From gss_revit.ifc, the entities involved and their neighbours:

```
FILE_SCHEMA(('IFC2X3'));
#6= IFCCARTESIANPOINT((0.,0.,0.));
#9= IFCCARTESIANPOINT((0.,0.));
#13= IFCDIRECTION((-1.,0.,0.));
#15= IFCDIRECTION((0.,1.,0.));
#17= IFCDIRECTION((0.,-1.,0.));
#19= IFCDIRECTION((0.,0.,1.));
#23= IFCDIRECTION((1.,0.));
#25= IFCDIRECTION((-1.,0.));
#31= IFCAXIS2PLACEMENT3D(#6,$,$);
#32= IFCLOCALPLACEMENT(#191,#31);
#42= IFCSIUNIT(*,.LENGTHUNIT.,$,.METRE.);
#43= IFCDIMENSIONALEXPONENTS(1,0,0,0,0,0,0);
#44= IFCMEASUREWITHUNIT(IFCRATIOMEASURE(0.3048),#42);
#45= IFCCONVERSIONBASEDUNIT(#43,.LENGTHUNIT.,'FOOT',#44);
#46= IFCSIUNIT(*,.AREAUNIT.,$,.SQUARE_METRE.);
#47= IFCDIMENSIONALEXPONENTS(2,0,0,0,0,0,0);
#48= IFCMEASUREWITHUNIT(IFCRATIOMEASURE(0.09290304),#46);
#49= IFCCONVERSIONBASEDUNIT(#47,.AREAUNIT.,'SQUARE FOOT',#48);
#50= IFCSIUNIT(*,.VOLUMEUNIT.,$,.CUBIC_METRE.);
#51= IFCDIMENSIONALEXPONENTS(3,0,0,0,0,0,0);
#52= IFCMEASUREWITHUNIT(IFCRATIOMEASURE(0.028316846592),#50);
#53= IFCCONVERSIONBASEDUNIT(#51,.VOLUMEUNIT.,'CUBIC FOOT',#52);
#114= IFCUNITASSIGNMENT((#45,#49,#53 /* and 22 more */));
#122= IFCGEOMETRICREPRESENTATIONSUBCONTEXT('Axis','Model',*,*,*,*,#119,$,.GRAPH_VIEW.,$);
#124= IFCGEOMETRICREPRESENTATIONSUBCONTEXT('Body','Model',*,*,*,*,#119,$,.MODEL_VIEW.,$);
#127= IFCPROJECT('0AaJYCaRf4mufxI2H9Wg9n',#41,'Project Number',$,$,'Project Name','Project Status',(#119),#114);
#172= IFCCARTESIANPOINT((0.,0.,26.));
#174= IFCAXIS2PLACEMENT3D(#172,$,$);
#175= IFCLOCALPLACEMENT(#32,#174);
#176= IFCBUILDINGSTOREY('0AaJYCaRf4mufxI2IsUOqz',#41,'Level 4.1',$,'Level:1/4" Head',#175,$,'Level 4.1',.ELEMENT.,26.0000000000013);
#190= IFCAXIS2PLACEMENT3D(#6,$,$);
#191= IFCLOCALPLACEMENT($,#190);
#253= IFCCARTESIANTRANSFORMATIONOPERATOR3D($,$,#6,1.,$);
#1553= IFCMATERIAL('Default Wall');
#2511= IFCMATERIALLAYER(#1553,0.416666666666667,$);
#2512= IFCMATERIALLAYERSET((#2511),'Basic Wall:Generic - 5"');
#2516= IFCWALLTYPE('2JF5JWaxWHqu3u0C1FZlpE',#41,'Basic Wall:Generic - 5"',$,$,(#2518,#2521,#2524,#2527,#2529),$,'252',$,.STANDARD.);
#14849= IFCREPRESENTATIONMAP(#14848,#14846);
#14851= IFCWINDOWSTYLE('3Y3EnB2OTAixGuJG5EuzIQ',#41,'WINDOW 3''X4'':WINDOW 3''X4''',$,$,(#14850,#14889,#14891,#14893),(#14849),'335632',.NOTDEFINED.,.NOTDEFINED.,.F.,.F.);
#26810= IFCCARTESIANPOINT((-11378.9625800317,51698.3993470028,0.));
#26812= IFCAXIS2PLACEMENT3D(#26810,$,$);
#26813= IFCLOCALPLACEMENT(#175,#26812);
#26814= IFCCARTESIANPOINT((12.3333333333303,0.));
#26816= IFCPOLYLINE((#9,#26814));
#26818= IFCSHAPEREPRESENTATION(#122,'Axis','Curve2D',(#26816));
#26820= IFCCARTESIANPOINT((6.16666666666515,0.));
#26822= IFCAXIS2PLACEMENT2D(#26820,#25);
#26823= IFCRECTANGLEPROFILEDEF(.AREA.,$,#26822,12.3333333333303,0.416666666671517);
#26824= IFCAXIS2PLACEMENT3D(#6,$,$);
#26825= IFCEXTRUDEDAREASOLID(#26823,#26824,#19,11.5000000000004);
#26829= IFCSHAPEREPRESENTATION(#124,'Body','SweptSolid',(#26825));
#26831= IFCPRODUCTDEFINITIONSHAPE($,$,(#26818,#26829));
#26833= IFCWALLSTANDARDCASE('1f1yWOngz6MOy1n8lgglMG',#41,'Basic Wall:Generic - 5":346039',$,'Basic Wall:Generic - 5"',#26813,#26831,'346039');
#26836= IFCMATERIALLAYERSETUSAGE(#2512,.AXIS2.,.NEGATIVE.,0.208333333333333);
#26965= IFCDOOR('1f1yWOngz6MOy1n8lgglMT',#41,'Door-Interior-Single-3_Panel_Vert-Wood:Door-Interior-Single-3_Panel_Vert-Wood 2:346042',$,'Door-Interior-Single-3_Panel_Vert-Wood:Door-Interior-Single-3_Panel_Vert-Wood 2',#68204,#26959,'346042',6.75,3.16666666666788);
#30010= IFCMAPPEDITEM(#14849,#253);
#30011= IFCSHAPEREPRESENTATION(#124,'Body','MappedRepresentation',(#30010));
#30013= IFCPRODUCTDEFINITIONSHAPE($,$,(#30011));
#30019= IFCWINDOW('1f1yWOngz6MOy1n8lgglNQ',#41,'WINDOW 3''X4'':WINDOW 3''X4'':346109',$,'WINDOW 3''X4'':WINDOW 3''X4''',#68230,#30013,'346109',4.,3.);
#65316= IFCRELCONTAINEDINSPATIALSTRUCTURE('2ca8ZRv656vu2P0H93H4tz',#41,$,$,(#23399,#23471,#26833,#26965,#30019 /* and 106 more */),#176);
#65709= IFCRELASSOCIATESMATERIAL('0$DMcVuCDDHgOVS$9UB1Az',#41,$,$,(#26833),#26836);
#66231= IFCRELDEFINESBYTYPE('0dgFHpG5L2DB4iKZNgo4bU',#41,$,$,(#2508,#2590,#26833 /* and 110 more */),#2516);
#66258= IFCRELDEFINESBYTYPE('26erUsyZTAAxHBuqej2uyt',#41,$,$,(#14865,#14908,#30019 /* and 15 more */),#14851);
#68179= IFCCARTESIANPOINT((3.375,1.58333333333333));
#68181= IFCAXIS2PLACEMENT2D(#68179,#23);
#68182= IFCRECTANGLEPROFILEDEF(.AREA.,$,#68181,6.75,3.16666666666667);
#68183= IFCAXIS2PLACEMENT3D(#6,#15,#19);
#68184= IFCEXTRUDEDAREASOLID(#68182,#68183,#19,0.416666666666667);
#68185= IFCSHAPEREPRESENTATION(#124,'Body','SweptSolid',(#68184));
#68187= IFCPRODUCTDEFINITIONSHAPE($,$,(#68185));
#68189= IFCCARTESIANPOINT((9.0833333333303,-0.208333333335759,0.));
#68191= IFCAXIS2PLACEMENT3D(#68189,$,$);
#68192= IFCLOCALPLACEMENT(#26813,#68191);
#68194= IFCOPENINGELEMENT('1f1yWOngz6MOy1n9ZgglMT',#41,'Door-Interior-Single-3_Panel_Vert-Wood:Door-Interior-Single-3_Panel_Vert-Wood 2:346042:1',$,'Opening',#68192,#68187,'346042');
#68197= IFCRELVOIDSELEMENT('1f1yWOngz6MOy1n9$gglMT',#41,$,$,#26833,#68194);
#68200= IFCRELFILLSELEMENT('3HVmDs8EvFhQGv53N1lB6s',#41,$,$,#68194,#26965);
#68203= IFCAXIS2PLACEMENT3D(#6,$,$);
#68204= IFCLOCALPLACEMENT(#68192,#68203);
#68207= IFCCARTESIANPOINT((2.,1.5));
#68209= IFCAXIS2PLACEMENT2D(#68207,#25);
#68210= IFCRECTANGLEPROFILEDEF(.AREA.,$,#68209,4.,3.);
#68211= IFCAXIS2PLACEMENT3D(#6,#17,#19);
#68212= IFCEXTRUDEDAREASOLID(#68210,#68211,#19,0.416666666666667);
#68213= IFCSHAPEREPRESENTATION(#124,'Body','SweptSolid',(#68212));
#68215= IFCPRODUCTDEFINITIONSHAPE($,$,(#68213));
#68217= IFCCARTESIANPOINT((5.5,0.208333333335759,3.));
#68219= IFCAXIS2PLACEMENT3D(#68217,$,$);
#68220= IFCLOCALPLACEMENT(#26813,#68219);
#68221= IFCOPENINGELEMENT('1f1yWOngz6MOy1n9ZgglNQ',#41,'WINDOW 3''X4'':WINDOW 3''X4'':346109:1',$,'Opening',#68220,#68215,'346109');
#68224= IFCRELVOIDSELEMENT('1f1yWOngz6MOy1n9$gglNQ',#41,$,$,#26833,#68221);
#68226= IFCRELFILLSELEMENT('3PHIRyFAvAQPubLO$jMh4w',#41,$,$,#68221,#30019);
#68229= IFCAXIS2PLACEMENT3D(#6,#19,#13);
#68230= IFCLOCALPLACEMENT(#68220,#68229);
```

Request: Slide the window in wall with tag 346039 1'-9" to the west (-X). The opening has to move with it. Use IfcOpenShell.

```python
import ifcopenshell
import ifcopenshell.api.geometry
import ifcopenshell.util.placement
import ifcopenshell.util.unit

model = ifcopenshell.open("gss_revit.ifc")
unit_scale = ifcopenshell.util.unit.calculate_unit_scale(model)

window = model.by_guid("1f1yWOngz6MOy1n8lgglNQ")
opening = window.FillsVoids[0].RelatingOpeningElement
wall = opening.VoidsElements[0].RelatingBuildingElement

wall_matrix = ifcopenshell.util.placement.get_local_placement(wall.ObjectPlacement)
shift = wall_matrix[:3, 0] * -21 * 0.0254 / unit_scale
before = ifcopenshell.util.placement.get_local_placement(window.ObjectPlacement)[:3, 3].copy()

# The window is placed relative to its opening, so it follows when the opening moves.
matrix = ifcopenshell.util.placement.get_local_placement(opening.ObjectPlacement)
matrix[:3, 3] += shift
ifcopenshell.api.geometry.edit_object_placement(
    model, product=opening, matrix=matrix, is_si=False, should_transform_children=True
)

after = ifcopenshell.util.placement.get_local_placement(window.ObjectPlacement)[:3, 3]
print("window moved by", (after - before).round(3) + 0.0)

model.write("gss_revit_rev.ifc")
```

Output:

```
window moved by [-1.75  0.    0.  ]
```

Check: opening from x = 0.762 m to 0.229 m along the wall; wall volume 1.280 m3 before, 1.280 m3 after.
